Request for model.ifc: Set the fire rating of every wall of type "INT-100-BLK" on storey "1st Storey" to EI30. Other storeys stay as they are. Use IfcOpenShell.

First a look at what the model holds.

```python
import ifcopenshell
import ifcopenshell.util.element

model = ifcopenshell.open("model.ifc")
print(model.schema)
storey = next(s for s in model.by_type("IfcBuildingStorey") if s.Name == "1st Storey")
walls = [e for e in ifcopenshell.util.element.get_decomposition(storey) if e.is_a("IfcWall")]
seen = {}
for e in walls:
    element_type = ifcopenshell.util.element.get_type(e)
    key = (element_type.Name if element_type != e and element_type else None, ifcopenshell.util.element.get_pset(e, "Pset_WallCommon", "FireRating"))
    seen[key] = seen.get(key, 0) + 1
for (name, value), count in sorted(seen.items(), key=str):
    print(count, "x", name, "|", value)
```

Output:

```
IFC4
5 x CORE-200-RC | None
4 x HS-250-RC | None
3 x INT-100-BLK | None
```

```python
import ifcopenshell
import ifcopenshell.api.pset
import ifcopenshell.util.element

model = ifcopenshell.open("model.ifc")

storey = next(s for s in model.by_type("IfcBuildingStorey") if s.Name == "1st Storey")
walls = [e for e in ifcopenshell.util.element.get_decomposition(storey) if e.is_a("IfcWall")]

count = 0
for e in walls:
    element_type = ifcopenshell.util.element.get_type(e)
    if element_type in (None, e) or element_type.Name != "INT-100-BLK":
        continue
    # add_pset returns the element's existing set when there is one.
    pset = ifcopenshell.api.pset.add_pset(model, product=e, name="Pset_WallCommon")
    ifcopenshell.api.pset.edit_pset(model, pset=pset, properties={"FireRating": "EI30"})
    count += 1

print(count, "walls updated")

model.write("model_rev.ifc")
```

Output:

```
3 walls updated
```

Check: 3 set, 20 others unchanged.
